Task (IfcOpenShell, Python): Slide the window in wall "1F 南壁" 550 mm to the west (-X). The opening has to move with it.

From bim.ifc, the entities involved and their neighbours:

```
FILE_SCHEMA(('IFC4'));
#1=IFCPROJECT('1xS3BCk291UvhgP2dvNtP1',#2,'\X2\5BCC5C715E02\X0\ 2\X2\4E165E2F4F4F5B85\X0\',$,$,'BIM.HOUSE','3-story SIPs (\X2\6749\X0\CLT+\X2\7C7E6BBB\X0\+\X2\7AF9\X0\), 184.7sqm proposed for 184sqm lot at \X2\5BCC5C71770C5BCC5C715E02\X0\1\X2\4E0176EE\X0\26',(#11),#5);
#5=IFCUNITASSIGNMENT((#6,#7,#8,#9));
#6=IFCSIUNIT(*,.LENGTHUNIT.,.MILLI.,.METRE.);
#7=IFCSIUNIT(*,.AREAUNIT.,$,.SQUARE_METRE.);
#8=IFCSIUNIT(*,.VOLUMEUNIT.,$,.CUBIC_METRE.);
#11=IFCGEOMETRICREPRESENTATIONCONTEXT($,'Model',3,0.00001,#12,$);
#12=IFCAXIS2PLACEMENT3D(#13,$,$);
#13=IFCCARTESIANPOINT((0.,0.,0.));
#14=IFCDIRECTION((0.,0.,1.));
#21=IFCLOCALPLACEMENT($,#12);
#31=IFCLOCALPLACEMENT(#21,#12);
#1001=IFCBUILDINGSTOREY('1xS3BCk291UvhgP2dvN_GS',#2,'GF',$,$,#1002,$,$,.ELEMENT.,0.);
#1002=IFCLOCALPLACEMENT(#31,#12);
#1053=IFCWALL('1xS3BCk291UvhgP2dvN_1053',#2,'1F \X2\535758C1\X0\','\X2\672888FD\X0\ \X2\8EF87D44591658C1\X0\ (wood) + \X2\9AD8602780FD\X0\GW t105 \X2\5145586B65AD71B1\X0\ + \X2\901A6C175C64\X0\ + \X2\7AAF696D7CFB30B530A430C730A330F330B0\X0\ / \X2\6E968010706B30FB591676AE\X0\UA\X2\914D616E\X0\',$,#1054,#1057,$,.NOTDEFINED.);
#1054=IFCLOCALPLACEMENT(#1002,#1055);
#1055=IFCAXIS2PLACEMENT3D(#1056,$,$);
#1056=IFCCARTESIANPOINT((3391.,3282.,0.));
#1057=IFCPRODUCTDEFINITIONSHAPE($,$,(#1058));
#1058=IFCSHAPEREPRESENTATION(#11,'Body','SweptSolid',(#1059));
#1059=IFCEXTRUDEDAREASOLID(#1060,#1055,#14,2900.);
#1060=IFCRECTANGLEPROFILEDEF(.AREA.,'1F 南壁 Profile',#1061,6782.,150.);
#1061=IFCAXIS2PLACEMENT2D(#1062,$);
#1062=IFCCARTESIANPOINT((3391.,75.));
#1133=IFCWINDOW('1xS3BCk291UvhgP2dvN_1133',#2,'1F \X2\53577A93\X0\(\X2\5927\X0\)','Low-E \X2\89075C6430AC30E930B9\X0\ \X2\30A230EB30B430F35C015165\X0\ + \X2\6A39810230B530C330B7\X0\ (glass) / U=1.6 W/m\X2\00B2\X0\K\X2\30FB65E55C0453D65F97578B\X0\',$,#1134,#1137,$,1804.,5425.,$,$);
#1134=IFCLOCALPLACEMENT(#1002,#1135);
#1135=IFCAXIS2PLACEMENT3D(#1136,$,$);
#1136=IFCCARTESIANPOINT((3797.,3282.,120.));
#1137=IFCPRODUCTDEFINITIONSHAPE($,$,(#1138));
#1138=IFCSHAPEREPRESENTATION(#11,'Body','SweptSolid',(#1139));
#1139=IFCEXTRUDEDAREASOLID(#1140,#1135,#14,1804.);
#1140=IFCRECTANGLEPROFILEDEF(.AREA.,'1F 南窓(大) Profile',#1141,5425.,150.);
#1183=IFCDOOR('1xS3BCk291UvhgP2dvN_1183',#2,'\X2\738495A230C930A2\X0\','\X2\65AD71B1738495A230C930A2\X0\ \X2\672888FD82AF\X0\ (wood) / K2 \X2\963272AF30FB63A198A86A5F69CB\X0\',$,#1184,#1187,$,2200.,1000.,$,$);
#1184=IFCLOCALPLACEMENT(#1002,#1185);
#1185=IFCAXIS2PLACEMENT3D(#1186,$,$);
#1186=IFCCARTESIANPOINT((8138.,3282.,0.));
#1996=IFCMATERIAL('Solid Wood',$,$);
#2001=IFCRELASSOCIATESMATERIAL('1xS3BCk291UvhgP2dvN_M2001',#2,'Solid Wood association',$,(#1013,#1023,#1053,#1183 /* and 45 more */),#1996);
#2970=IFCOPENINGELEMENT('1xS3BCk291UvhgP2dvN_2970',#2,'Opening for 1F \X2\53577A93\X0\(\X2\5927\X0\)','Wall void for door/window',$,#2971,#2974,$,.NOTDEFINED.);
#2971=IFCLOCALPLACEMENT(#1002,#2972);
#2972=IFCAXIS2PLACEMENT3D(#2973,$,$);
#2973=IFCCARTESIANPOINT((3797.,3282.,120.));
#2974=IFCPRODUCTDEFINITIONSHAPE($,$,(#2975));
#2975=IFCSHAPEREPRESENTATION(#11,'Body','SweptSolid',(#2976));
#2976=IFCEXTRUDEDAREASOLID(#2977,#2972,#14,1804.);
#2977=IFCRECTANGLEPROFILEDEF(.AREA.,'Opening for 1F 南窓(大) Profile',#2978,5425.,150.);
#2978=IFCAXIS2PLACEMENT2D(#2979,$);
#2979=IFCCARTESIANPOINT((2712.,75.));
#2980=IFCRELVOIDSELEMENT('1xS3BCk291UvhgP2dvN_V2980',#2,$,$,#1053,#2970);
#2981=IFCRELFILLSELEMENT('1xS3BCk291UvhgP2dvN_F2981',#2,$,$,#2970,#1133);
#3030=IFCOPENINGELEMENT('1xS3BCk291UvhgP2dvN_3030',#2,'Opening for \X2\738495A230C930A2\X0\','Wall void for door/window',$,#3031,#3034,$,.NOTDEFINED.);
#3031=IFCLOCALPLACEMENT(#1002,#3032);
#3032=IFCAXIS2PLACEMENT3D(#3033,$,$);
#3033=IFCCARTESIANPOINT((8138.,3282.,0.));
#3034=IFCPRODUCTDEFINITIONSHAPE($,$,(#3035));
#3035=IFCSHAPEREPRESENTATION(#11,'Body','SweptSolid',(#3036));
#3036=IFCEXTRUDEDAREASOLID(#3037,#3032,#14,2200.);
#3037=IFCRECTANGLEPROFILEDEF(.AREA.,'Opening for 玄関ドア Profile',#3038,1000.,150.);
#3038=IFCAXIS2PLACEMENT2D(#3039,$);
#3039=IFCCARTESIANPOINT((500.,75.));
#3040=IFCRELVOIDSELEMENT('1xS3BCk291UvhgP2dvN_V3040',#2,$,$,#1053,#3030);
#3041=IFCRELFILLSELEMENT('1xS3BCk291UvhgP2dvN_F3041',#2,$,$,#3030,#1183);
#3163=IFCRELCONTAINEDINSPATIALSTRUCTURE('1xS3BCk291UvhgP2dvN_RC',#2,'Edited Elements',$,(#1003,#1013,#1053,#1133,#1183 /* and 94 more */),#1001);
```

```python
import ifcopenshell
import ifcopenshell.api.geometry
import ifcopenshell.util.placement
import ifcopenshell.util.unit

model = ifcopenshell.open("bim.ifc")
unit_scale = ifcopenshell.util.unit.calculate_unit_scale(model)

window = model.by_id(1133)
opening = window.FillsVoids[0].RelatingOpeningElement
wall = opening.VoidsElements[0].RelatingBuildingElement

wall_matrix = ifcopenshell.util.placement.get_local_placement(wall.ObjectPlacement)
shift = wall_matrix[:3, 0] * -0.55 / unit_scale
before = ifcopenshell.util.placement.get_local_placement(window.ObjectPlacement)[:3, 3].copy()

# The window is not placed relative to its opening, so move both.
for product in (opening, window):
    matrix = ifcopenshell.util.placement.get_local_placement(product.ObjectPlacement)
    matrix[:3, 3] += shift
    ifcopenshell.api.geometry.edit_object_placement(model, product=product, matrix=matrix, is_si=False)

after = ifcopenshell.util.placement.get_local_placement(window.ObjectPlacement)[:3, 3]
print("window moved by", (after - before).round(3) + 0.0)

model.write("bim-out.ifc")
```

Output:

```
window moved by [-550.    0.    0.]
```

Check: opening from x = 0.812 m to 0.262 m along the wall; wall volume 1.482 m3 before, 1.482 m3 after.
